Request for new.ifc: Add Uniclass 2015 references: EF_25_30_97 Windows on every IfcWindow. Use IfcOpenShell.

First a look at what the model holds.

```python
import ifcopenshell

model = ifcopenshell.open("new.ifc")
print(model.schema)
print("classifications:", [c.Name for c in model.by_type("IfcClassification")])
for ifc_class in ("IfcDoor", "IfcRoof", "IfcStair", "IfcWall", "IfcWindow"):
    print(ifc_class, len(model.by_type(ifc_class)))
```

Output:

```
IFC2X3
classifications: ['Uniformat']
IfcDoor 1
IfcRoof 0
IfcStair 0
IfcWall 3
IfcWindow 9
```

```python
import ifcopenshell
import ifcopenshell.api.classification

model = ifcopenshell.open("new.ifc")

# IFC2X3 requires Source and Edition and has no link from the project to the system.
system = model.create_entity("IfcClassification", Source="NBS", Edition="2015", Name="Uniclass 2015")

codes = {
    "IfcWindow": ("EF_25_30_97", "Windows"),
}
for ifc_class, (code, name) in codes.items():
    products = model.by_type(ifc_class)
    ifcopenshell.api.classification.add_reference(
        model, products=products, classification=system, identification=code, name=name
    )
    print(code, len(products))

model.write("new_v2.ifc")
```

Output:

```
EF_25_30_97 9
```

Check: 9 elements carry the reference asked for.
